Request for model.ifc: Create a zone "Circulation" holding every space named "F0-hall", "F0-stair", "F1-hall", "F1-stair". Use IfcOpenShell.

First a look at what the model holds.

```python
import ifcopenshell

model = ifcopenshell.open("model.ifc")
print(model.schema)
seen = {}
for space in model.by_type("IfcSpace"):
    seen[space.LongName] = seen.get(space.LongName, 0) + 1
for name, count in sorted(seen.items(), key=str):
    print(count, "x", name)
print("zones:", [z.Name for z in model.by_type("IfcZone")][:20])
```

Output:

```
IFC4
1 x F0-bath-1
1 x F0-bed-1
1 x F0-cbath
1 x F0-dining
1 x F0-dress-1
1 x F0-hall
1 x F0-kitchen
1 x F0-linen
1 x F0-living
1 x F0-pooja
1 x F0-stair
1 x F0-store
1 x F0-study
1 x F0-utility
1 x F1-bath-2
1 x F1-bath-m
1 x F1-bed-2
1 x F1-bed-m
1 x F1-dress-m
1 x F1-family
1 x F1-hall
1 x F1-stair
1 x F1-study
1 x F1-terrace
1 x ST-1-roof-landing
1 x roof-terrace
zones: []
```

```python
import ifcopenshell
import ifcopenshell.api.group
import ifcopenshell.api.root

model = ifcopenshell.open("model.ifc")

names = {"F0-hall", "F0-stair", "F1-hall", "F1-stair"}
spaces = [s for s in model.by_type("IfcSpace") if s.LongName in names]

zone = ifcopenshell.api.root.create_entity(model, ifc_class="IfcZone", name="Circulation")
ifcopenshell.api.group.assign_group(model, products=spaces, group=zone)
print(len(spaces), "spaces in", zone.Name)

model.write("model_rev.ifc")
```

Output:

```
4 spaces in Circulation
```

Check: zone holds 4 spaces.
